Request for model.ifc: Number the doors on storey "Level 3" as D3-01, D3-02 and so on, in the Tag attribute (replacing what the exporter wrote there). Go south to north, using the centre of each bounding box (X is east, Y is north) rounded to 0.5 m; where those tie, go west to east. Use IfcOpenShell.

First a look at what the model holds.

```python
import ifcopenshell
import ifcopenshell.util.element
import ifcopenshell.util.placement

model = ifcopenshell.open("model.ifc")
print(model.schema)
storey = next(s for s in model.by_type("IfcBuildingStorey") if s.Name == "Level 3")
doors = [e for e in ifcopenshell.util.element.get_decomposition(storey) if e.is_a("IfcDoor")]
for e in sorted(doors, key=lambda e: e.id()):
    origin = ifcopenshell.util.placement.get_local_placement(e.ObjectPlacement)[:3, 3]
    print(e.id(), e.Tag, e.Name, origin.round(2) + 0.0, sep=" | ")
```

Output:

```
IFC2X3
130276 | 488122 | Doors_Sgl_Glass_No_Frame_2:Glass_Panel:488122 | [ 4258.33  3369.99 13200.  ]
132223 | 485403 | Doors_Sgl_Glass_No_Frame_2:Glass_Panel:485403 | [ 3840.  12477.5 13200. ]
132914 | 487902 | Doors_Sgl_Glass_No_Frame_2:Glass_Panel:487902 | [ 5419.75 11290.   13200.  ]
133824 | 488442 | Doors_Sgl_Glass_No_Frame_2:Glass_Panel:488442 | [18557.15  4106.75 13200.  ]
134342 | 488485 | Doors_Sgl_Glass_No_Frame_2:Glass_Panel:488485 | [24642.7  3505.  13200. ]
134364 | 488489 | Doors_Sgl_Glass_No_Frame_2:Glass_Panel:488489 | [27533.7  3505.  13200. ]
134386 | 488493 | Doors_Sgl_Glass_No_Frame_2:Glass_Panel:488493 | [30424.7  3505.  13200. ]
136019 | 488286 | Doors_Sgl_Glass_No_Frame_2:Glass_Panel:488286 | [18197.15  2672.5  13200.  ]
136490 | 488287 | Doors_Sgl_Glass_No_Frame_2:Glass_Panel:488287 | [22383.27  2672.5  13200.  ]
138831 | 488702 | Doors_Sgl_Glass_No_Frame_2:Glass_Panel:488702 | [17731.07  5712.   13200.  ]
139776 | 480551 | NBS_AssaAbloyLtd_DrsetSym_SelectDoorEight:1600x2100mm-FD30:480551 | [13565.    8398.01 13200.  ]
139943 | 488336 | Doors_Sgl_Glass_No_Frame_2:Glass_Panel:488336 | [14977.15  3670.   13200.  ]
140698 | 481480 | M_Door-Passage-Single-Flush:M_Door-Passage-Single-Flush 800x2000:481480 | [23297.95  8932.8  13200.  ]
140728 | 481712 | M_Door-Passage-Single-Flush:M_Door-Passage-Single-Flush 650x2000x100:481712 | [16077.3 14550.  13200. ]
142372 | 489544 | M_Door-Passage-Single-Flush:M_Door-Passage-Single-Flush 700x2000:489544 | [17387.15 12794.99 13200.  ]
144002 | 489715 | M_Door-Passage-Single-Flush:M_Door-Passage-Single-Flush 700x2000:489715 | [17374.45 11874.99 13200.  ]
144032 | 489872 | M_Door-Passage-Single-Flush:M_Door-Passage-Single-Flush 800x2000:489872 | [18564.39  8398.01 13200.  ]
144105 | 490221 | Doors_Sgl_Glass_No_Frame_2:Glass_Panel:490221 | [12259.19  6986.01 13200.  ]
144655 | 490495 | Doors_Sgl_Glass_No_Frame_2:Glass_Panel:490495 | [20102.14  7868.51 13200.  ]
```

```python
import ifcopenshell
import ifcopenshell.geom
import ifcopenshell.util.element
import ifcopenshell.util.shape

model = ifcopenshell.open("model.ifc")
settings = ifcopenshell.geom.settings()
settings.set("use-world-coords", True)


def centre(element):
    shape = ifcopenshell.geom.create_shape(settings, element)
    return ifcopenshell.util.shape.get_bbox_centroid(shape.geometry)


storey = next(s for s in model.by_type("IfcBuildingStorey") if s.Name == "Level 3")
doors = [e for e in ifcopenshell.util.element.get_decomposition(storey) if e.is_a("IfcDoor")]

# Insertion points can sit at a corner or the storey origin, so sort by the geometry (in metres).
centres = {e: centre(e) for e in doors}
doors.sort(key=lambda e: (round(centres[e][1] / 0.5), centres[e][0]))

for i, e in enumerate(doors, start=1):
    number = f"D3-{i:02d}"
    e.Tag = number
    print(e.id(), number)

model.write("model-out.ifc")
```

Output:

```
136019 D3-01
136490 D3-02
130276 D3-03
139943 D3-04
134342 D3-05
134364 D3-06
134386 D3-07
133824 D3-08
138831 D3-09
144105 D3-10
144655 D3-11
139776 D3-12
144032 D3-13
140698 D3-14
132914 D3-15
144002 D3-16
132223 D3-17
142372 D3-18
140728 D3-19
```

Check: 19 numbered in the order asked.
